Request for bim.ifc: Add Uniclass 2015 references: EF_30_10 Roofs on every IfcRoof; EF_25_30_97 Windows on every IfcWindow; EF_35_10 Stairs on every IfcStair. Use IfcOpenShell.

First a look at what the model holds.

```python
import ifcopenshell

model = ifcopenshell.open("bim.ifc")
print(model.schema)
print("classifications:", [c.Name for c in model.by_type("IfcClassification")])
for ifc_class in ("IfcDoor", "IfcRoof", "IfcStair", "IfcWall", "IfcWindow"):
    print(ifc_class, len(model.by_type(ifc_class)))
```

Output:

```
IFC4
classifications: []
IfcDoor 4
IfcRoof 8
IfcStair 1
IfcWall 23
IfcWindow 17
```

```python
import ifcopenshell
import ifcopenshell.api.classification

model = ifcopenshell.open("bim.ifc")

system = ifcopenshell.api.classification.add_classification(model, classification="Uniclass 2015")

codes = {
    "IfcRoof": ("EF_30_10", "Roofs"),
    "IfcWindow": ("EF_25_30_97", "Windows"),
    "IfcStair": ("EF_35_10", "Stairs"),
}
for ifc_class, (code, name) in codes.items():
    products = model.by_type(ifc_class)
    ifcopenshell.api.classification.add_reference(
        model, products=products, classification=system, identification=code, name=name
    )
    print(code, len(products))

model.write("bim_updated.ifc")
```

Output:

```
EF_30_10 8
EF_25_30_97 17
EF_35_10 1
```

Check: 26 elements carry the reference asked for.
